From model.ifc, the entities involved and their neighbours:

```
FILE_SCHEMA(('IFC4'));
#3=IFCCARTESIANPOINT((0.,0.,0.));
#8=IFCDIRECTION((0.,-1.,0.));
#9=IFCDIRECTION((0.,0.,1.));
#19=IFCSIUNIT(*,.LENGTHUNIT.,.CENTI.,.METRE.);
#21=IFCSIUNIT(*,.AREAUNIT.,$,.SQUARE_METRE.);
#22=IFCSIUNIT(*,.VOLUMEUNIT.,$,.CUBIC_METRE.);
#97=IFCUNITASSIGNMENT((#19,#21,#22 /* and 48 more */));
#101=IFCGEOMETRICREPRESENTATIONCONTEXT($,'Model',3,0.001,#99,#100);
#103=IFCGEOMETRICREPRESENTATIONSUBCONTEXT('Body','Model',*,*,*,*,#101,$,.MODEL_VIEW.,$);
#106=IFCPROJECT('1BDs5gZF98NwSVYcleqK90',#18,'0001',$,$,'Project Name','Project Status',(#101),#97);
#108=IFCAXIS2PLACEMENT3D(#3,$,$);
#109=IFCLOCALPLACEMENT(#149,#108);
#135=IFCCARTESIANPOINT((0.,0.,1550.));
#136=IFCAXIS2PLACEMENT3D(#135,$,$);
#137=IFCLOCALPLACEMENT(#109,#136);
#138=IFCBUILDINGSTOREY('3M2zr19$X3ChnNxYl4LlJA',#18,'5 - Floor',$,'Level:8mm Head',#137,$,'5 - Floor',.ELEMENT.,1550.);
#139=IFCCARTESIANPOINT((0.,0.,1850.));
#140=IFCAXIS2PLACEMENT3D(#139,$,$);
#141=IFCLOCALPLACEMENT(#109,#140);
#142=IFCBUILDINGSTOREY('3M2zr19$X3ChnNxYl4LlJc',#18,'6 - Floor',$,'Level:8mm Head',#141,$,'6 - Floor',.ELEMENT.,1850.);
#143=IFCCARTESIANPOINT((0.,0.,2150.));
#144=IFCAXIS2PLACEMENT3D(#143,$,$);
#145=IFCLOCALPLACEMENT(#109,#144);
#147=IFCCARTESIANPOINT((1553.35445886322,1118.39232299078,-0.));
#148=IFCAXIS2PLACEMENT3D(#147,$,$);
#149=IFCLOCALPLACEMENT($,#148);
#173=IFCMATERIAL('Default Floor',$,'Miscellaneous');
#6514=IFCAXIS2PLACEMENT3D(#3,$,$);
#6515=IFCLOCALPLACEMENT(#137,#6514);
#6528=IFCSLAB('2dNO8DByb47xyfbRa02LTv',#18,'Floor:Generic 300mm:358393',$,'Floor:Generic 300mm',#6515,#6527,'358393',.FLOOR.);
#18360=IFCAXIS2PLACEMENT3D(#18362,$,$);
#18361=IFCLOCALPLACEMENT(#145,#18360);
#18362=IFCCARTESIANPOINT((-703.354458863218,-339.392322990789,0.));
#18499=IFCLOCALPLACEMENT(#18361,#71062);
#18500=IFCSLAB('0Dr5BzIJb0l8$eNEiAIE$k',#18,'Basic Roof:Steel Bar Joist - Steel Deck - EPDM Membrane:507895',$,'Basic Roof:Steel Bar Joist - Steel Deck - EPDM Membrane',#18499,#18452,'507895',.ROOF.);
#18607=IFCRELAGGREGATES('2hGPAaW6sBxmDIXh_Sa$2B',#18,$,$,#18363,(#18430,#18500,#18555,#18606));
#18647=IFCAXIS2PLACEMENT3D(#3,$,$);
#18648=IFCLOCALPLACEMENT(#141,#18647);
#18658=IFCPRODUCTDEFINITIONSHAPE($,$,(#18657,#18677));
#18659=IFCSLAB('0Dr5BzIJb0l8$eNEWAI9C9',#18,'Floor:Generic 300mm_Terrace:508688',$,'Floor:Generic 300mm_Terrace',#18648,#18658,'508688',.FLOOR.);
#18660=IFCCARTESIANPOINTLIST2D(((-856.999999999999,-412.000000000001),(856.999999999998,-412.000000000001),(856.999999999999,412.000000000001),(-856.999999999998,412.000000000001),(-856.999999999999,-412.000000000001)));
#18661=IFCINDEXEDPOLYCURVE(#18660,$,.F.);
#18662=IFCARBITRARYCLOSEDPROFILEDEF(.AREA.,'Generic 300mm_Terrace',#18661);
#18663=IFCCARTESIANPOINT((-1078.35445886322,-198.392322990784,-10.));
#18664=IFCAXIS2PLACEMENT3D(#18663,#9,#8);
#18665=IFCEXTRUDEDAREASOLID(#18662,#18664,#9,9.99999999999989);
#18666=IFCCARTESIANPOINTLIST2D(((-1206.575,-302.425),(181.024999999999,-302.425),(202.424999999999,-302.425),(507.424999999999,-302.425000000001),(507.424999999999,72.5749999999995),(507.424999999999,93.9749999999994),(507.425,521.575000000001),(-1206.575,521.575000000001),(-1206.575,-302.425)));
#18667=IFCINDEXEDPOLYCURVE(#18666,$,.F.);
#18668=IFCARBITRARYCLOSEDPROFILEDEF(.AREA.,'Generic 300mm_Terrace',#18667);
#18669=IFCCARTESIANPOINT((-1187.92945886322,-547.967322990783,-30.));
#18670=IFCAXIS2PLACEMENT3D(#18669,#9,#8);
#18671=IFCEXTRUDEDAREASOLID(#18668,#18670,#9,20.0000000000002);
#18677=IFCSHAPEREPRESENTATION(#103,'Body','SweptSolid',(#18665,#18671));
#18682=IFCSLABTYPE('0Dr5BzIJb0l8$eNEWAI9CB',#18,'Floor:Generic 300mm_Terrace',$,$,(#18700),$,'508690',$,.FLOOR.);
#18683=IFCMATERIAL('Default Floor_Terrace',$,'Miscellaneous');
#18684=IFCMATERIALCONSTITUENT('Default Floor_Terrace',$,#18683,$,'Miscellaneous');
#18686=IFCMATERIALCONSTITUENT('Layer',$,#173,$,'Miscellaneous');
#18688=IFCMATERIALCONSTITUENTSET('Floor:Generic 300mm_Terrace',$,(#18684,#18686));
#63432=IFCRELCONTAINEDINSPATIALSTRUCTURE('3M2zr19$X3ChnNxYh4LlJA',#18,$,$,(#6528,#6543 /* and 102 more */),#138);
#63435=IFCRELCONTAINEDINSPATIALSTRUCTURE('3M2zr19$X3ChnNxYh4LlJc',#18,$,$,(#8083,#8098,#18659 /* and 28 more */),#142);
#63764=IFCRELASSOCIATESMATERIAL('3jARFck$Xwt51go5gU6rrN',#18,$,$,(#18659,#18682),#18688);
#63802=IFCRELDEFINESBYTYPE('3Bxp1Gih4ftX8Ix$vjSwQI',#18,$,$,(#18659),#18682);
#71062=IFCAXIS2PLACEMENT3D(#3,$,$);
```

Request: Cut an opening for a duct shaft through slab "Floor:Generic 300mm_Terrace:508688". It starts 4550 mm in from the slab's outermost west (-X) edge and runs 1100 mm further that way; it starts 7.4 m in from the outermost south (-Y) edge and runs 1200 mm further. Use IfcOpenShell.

```python
import numpy as np
import ifcopenshell
import ifcopenshell.api.feature
import ifcopenshell.api.geometry
import ifcopenshell.api.root
import ifcopenshell.geom
import ifcopenshell.util.placement
import ifcopenshell.util.representation
import ifcopenshell.util.shape
import ifcopenshell.util.unit

model = ifcopenshell.open("model.ifc")
unit_scale = ifcopenshell.util.unit.calculate_unit_scale(model)
settings = ifcopenshell.geom.settings()


def volume(element):
    """Net volume in cubic metres, openings subtracted."""
    shape = ifcopenshell.geom.create_shape(settings, element)
    return ifcopenshell.util.shape.get_volume(shape.geometry)


slab = model.by_guid("0Dr5BzIJb0l8$eNEWAI9C9")
before = volume(slab)

# Extent in the slab's own axes, in metres. The edges named are its -X and -Y sides.
slab_shape = ifcopenshell.geom.create_shape(settings, slab)
vertices = ifcopenshell.util.shape.get_vertices(slab_shape.geometry)
x_min, y_min, bottom = vertices.min(axis=0)
top = vertices[:, 2].max()

opening = ifcopenshell.api.root.create_entity(model, ifc_class="IfcOpeningElement", name="Duct shaft opening", predefined_type="OPENING")
context = ifcopenshell.util.representation.get_context(model, "Model", "Body", "MODEL_VIEW")
width, depth = 1.1, 1.2
outline = [(0.0, 0.0), (width, 0.0), (width, depth), (0.0, depth), (0.0, 0.0)]
# Overshoot both faces by 50 mm so the cut is clean.
shape = ifcopenshell.api.geometry.add_slab_representation(
    model, context=context, depth=top - bottom + 0.1, polyline=outline
)
ifcopenshell.api.geometry.assign_representation(model, product=opening, representation=shape)

matrix = ifcopenshell.util.placement.get_local_placement(slab.ObjectPlacement)
matrix[:, 3] = matrix @ np.append(np.array([x_min + 4.55, y_min + 7.4, bottom - 0.05]) / unit_scale, 1.0)
ifcopenshell.api.geometry.edit_object_placement(model, product=opening, matrix=matrix, is_si=False)
ifcopenshell.api.feature.add_feature(model, feature=opening, element=slab)

after = volume(slab)

print(f"slab volume {before:.3f} -> {after:.3f} m3")

model.write("model_rev.ifc")
```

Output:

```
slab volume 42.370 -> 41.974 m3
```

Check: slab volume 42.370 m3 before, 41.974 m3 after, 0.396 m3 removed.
